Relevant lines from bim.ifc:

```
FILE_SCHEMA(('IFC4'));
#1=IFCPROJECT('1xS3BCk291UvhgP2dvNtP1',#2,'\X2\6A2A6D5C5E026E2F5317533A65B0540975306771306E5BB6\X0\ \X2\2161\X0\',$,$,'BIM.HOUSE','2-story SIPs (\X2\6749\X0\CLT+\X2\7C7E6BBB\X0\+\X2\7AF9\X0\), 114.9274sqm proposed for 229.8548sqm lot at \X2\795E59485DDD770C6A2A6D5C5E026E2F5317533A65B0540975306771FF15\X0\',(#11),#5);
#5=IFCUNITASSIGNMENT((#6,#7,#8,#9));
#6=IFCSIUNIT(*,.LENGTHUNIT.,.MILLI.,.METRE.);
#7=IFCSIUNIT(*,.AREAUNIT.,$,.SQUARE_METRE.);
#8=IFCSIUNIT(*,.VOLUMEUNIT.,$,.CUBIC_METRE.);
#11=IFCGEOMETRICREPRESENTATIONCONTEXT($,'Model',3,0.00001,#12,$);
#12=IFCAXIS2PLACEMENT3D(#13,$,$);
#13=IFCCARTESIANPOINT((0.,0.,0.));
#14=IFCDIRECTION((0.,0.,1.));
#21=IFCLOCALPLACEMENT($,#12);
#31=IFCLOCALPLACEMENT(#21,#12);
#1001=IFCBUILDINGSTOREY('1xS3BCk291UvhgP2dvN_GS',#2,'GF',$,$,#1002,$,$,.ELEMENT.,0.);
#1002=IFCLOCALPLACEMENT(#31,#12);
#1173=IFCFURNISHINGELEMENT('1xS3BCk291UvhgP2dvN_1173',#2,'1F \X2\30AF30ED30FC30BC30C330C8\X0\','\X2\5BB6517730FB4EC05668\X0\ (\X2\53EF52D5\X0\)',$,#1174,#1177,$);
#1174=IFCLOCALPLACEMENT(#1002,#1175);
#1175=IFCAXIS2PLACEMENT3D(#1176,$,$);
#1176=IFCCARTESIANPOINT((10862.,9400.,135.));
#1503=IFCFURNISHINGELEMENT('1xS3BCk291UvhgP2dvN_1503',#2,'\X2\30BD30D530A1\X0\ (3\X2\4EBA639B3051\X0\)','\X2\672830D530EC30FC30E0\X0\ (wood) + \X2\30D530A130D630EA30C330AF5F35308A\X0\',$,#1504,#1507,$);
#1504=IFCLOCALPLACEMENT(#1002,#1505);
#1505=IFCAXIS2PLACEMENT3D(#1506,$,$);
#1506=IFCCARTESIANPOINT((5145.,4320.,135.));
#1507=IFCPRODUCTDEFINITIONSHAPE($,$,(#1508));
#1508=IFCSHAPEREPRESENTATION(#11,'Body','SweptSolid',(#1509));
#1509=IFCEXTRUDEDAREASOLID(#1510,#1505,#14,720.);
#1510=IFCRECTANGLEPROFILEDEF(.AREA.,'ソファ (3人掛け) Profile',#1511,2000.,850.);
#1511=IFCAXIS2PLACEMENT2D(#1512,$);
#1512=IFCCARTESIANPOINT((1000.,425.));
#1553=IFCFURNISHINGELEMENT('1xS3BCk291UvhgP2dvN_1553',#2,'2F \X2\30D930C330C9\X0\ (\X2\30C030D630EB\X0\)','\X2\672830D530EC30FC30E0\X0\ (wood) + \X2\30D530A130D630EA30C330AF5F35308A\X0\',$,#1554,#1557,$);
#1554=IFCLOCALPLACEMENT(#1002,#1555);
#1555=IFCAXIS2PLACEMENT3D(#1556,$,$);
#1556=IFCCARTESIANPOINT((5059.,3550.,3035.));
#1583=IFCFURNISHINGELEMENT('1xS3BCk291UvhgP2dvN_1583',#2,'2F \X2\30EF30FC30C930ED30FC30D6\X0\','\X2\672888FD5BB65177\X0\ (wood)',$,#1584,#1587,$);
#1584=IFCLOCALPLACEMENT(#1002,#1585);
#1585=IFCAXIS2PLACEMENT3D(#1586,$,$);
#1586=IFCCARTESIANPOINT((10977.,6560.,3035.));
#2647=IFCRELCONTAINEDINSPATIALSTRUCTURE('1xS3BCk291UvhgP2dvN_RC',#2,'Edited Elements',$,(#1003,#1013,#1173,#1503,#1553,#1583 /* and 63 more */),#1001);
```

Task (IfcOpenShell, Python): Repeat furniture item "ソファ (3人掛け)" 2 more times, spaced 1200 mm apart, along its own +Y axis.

```python
import ifcopenshell
import ifcopenshell.api.geometry
import ifcopenshell.api.root
import ifcopenshell.util.element
import ifcopenshell.util.placement
import ifcopenshell.util.unit

model = ifcopenshell.open("bim.ifc")
unit_scale = ifcopenshell.util.unit.calculate_unit_scale(model)


def reuse_history(source, copy):
    """copy_class also copies each property set's owner history, people and application; keep the originals."""
    for rel in copy.IsDefinedBy:
        if rel.is_a("IfcRelDefinesByProperties") and (history := rel.RelatingPropertyDefinition.OwnerHistory):
            rel.RelatingPropertyDefinition.OwnerHistory = source.OwnerHistory
            ifcopenshell.util.element.remove_deep2(model, history)


source = model.by_guid("1xS3BCk291UvhgP2dvN_1503")
base = ifcopenshell.util.placement.get_local_placement(source.ObjectPlacement)
step = base[:3, 1] * 1.2 / unit_scale

for i in range(1, 3):
    copy = ifcopenshell.api.root.copy_class(model, product=source)
    copy.Representation = ifcopenshell.util.element.copy_deep(
        model, source.Representation, exclude=["IfcGeometricRepresentationContext", "IfcRepresentationMap"]
    )
    reuse_history(source, copy)
    matrix = base.copy()
    matrix[:3, 3] += i * step
    print("added at", matrix[:3, 3].round(3) + 0.0)
    ifcopenshell.api.geometry.edit_object_placement(model, product=copy, matrix=matrix, is_si=False)

model.write("bim_rev.ifc")
```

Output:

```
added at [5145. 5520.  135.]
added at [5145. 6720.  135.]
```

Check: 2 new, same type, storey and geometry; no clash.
